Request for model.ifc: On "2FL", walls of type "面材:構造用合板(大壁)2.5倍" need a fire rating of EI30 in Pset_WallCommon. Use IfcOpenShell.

First a look at what the model holds.

```python
import ifcopenshell
import ifcopenshell.util.element

model = ifcopenshell.open("model.ifc")
print(model.schema)
storey = next(s for s in model.by_type("IfcBuildingStorey") if s.Name == "2FL")
walls = [e for e in ifcopenshell.util.element.get_decomposition(storey) if e.is_a("IfcWall")]
seen = {}
for e in walls:
    element_type = ifcopenshell.util.element.get_type(e)
    key = (element_type.Name if element_type != e and element_type else None, ifcopenshell.util.element.get_pset(e, "Pset_WallCommon", "FireRating"))
    seen[key] = seen.get(key, 0) + 1
for (name, value), count in sorted(seen.items(), key=str):
    print(count, "x", name, "|", value)
```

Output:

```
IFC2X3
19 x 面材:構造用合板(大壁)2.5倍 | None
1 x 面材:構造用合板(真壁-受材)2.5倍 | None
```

```python
import ifcopenshell
import ifcopenshell.api.pset
import ifcopenshell.util.element

model = ifcopenshell.open("model.ifc")

storey = next(s for s in model.by_type("IfcBuildingStorey") if s.Name == "2FL")
walls = [e for e in ifcopenshell.util.element.get_decomposition(storey) if e.is_a("IfcWall")]

count = 0
for e in walls:
    element_type = ifcopenshell.util.element.get_type(e)
    if element_type in (None, e) or element_type.Name != "面材:構造用合板(大壁)2.5倍":
        continue
    # add_pset returns the element's existing set when there is one.
    pset = ifcopenshell.api.pset.add_pset(model, product=e, name="Pset_WallCommon")
    ifcopenshell.api.pset.edit_pset(model, pset=pset, properties={"FireRating": "EI30"})
    count += 1

print(count, "walls updated")

model.write("model_updated.ifc")
```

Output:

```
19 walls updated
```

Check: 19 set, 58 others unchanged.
